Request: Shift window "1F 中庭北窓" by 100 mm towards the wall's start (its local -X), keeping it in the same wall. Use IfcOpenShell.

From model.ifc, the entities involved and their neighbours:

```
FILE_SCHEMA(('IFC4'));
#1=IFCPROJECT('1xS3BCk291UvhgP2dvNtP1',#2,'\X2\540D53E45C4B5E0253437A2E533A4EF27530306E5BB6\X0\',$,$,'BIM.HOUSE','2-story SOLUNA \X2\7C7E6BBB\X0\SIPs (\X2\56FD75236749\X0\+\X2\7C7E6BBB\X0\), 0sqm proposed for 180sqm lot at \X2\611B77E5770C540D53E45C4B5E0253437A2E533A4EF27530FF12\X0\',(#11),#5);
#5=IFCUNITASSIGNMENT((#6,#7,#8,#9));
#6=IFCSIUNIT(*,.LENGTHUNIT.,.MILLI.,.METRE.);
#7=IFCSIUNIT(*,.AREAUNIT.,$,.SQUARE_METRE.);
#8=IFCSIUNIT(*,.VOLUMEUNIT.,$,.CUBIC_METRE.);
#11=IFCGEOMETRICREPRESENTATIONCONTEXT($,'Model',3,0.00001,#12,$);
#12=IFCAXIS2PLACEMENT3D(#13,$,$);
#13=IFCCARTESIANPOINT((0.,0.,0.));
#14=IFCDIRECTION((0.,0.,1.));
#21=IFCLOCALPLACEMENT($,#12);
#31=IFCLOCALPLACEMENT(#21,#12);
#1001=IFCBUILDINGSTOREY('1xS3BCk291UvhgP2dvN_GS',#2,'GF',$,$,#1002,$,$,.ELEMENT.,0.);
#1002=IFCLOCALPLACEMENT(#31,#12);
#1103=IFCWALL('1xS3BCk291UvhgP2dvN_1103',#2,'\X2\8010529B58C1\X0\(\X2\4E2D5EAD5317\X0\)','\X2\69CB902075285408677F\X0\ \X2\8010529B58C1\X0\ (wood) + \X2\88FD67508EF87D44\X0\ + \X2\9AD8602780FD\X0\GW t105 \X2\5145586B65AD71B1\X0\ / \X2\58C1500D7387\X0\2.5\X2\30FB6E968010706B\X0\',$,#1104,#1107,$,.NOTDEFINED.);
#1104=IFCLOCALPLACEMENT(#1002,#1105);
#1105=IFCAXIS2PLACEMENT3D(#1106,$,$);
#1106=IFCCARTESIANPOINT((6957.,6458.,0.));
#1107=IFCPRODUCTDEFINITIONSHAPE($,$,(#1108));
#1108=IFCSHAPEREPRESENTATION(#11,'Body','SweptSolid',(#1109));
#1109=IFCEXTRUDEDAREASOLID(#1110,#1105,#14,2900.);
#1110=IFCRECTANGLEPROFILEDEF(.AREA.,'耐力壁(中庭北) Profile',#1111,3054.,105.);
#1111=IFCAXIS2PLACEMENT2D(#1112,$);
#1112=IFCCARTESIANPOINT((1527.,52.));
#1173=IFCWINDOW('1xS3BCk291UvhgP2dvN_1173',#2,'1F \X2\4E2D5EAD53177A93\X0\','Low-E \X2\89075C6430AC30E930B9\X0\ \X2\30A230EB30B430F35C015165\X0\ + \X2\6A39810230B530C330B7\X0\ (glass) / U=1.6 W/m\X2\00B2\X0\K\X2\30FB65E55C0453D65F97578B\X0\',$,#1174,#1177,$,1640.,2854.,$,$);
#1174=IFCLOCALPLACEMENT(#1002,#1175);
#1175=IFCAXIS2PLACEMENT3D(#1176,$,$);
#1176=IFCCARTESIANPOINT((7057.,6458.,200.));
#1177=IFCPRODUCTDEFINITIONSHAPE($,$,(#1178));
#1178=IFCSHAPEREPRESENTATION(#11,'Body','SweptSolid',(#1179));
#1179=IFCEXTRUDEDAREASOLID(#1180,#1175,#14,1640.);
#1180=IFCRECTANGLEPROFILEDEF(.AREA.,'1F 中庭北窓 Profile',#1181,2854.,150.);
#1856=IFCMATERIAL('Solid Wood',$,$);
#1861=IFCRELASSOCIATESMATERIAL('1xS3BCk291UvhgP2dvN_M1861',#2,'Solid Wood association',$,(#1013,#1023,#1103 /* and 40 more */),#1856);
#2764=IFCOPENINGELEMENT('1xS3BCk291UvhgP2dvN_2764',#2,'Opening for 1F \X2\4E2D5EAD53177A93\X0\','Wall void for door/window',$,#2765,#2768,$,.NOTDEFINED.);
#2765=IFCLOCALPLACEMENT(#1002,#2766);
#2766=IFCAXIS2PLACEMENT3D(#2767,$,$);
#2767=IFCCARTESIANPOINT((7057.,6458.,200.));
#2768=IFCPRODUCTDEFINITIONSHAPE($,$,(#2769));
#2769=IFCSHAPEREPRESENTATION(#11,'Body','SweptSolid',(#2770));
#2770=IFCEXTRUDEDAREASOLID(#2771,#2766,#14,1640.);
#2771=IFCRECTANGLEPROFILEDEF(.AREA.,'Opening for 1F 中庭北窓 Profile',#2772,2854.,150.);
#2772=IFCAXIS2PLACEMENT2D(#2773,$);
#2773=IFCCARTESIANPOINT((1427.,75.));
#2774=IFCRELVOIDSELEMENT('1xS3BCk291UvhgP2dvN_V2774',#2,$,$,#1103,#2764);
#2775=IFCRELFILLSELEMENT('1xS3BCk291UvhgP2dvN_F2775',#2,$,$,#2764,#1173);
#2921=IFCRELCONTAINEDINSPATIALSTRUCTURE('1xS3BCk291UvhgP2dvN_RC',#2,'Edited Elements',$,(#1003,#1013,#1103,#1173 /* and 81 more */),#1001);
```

```python
import ifcopenshell
import ifcopenshell.api.geometry
import ifcopenshell.util.placement

model = ifcopenshell.open("model.ifc")

window = model.by_guid("1xS3BCk291UvhgP2dvN_1173")
opening = window.FillsVoids[0].RelatingOpeningElement
wall = opening.VoidsElements[0].RelatingBuildingElement

wall_matrix = ifcopenshell.util.placement.get_local_placement(wall.ObjectPlacement)
shift = wall_matrix[:3, 0] * -100.0
before = ifcopenshell.util.placement.get_local_placement(window.ObjectPlacement)[:3, 3].copy()

# The window is not placed relative to its opening, so move both.
for product in (opening, window):
    matrix = ifcopenshell.util.placement.get_local_placement(product.ObjectPlacement)
    matrix[:3, 3] += shift
    ifcopenshell.api.geometry.edit_object_placement(model, product=product, matrix=matrix, is_si=False)

after = ifcopenshell.util.placement.get_local_placement(window.ObjectPlacement)[:3, 3]
print("window moved by", (after - before).round(3) + 0.0)

model.write("model_edited.ifc")
```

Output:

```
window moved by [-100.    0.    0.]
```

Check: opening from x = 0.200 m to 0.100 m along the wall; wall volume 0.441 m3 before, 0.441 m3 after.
